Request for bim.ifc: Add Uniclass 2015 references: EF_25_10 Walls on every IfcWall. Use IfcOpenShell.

First a look at what the model holds.

```python
import ifcopenshell

model = ifcopenshell.open("bim.ifc")
print(model.schema)
print("classifications:", [c.Name for c in model.by_type("IfcClassification")])
for ifc_class in ("IfcDoor", "IfcRoof", "IfcStair", "IfcWall", "IfcWindow"):
    print(ifc_class, len(model.by_type(ifc_class)))
```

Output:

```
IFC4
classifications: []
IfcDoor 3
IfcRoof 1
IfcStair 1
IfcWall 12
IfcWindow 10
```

```python
import ifcopenshell
import ifcopenshell.api.classification

model = ifcopenshell.open("bim.ifc")

system = ifcopenshell.api.classification.add_classification(model, classification="Uniclass 2015")

codes = {
    "IfcWall": ("EF_25_10", "Walls"),
}
for ifc_class, (code, name) in codes.items():
    products = model.by_type(ifc_class)
    ifcopenshell.api.classification.add_reference(
        model, products=products, classification=system, identification=code, name=name
    )
    print(code, len(products))

model.write("bim_rev.ifc")
```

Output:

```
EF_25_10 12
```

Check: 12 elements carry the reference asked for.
